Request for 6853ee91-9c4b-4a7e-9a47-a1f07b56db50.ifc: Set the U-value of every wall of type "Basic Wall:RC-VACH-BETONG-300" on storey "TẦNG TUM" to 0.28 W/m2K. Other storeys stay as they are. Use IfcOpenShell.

First a look at what the model holds.

```python
import ifcopenshell
import ifcopenshell.util.element

model = ifcopenshell.open("6853ee91-9c4b-4a7e-9a47-a1f07b56db50.ifc")
print(model.schema)
storey = next(s for s in model.by_type("IfcBuildingStorey") if s.Name == "TẦNG TUM")
walls = [e for e in ifcopenshell.util.element.get_decomposition(storey) if e.is_a("IfcWall")]
seen = {}
for e in walls:
    element_type = ifcopenshell.util.element.get_type(e)
    key = (element_type.Name if element_type != e and element_type else None, ifcopenshell.util.element.get_pset(e, "Pset_WallCommon", "ThermalTransmittance"))
    seen[key] = seen.get(key, 0) + 1
for (name, value), count in sorted(seen.items(), key=str):
    print(count, "x", name, "|", value)
```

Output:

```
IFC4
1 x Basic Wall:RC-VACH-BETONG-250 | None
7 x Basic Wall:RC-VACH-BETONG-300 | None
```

```python
import ifcopenshell
import ifcopenshell.api.pset
import ifcopenshell.util.element

model = ifcopenshell.open("6853ee91-9c4b-4a7e-9a47-a1f07b56db50.ifc")

storey = next(s for s in model.by_type("IfcBuildingStorey") if s.Name == "TẦNG TUM")
walls = [e for e in ifcopenshell.util.element.get_decomposition(storey) if e.is_a("IfcWall")]

count = 0
for e in walls:
    element_type = ifcopenshell.util.element.get_type(e)
    if element_type in (None, e) or element_type.Name != "Basic Wall:RC-VACH-BETONG-300":
        continue
    # add_pset returns the element's existing set when there is one.
    pset = ifcopenshell.api.pset.add_pset(model, product=e, name="Pset_WallCommon")
    ifcopenshell.api.pset.edit_pset(model, pset=pset, properties={"ThermalTransmittance": 0.28})
    count += 1

print(count, "walls updated")

model.write("6853ee91-9c4b-4a7e-9a47-a1f07b56db50_edited.ifc")
```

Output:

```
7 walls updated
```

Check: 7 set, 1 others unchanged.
